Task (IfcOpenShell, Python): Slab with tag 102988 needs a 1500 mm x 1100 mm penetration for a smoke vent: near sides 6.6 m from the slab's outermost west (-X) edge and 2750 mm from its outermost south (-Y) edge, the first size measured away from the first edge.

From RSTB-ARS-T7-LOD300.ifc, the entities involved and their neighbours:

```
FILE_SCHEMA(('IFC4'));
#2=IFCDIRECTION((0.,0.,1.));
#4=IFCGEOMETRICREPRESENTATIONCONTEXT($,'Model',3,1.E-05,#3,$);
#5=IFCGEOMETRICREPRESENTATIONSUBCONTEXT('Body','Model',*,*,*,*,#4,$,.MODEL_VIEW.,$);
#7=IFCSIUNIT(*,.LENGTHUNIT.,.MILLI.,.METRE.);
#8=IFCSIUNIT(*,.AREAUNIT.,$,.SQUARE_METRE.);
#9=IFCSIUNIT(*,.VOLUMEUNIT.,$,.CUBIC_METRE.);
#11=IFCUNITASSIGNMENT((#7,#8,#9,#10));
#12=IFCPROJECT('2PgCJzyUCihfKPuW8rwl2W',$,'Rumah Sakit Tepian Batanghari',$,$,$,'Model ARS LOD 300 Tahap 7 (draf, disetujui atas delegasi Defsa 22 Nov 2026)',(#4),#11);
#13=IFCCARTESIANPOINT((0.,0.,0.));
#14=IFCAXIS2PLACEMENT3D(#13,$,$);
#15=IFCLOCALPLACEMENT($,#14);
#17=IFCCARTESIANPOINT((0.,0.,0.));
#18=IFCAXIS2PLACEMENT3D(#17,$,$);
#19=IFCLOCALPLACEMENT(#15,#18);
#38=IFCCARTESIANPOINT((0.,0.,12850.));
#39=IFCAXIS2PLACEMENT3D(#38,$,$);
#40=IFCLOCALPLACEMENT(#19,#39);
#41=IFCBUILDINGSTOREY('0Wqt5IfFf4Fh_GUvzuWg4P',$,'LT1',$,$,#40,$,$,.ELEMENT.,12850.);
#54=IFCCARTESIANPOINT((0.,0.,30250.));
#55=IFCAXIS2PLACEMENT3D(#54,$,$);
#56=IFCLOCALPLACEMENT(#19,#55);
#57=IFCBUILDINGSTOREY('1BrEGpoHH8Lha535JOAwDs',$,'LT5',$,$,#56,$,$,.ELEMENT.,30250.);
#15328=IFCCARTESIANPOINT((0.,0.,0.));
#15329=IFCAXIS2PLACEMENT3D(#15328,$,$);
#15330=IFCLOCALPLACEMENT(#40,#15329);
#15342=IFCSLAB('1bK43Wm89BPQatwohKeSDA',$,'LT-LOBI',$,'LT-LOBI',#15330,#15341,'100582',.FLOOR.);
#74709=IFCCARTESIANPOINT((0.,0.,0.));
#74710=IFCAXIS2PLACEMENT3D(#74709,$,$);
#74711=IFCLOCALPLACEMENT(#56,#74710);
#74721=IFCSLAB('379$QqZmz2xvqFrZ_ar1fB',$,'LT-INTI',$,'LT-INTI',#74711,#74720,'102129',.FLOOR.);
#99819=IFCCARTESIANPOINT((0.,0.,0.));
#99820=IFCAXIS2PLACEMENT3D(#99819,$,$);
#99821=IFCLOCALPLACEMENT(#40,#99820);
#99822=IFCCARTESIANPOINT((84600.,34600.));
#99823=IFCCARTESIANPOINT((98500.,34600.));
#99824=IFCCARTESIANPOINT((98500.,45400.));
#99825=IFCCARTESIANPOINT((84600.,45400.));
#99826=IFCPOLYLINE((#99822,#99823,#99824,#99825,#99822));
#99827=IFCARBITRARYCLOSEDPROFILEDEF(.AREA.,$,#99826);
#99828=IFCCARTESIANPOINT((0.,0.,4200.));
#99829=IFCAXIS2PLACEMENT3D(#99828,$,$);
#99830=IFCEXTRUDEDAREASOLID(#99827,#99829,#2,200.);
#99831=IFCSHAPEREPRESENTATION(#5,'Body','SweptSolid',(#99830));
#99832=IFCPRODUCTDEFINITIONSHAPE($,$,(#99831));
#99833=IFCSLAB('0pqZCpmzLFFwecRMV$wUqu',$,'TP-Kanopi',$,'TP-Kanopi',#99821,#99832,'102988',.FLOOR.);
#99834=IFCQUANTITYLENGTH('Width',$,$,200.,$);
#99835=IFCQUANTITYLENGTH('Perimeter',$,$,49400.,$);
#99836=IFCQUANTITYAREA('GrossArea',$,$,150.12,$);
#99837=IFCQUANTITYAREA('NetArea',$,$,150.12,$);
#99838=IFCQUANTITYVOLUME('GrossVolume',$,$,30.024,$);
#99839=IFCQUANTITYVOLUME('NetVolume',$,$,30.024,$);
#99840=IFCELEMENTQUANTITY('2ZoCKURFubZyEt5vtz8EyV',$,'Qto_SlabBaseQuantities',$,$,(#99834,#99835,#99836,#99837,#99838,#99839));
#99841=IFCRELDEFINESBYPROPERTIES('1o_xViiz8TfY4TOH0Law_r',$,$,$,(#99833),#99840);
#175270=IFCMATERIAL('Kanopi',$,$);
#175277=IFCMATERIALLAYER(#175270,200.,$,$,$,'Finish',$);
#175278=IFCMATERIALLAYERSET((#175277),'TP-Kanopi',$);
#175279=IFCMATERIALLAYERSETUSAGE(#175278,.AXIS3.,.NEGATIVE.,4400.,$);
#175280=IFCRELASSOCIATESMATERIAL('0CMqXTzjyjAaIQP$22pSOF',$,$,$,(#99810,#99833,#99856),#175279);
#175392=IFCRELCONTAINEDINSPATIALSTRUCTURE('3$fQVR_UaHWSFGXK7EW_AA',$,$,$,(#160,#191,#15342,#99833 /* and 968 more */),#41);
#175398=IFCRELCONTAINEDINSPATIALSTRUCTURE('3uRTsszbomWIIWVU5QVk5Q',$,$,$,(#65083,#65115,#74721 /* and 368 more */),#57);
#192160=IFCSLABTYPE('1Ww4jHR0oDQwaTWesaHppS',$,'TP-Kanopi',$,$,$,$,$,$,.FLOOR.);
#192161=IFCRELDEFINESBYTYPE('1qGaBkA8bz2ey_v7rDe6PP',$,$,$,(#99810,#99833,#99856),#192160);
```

```python
import numpy as np
import ifcopenshell
import ifcopenshell.api.feature
import ifcopenshell.api.geometry
import ifcopenshell.api.pset
import ifcopenshell.api.root
import ifcopenshell.geom
import ifcopenshell.util.element
import ifcopenshell.util.placement
import ifcopenshell.util.representation
import ifcopenshell.util.shape
import ifcopenshell.util.unit

model = ifcopenshell.open("RSTB-ARS-T7-LOD300.ifc")
unit_scale = ifcopenshell.util.unit.calculate_unit_scale(model)
area_scale = ifcopenshell.util.unit.calculate_unit_scale(model, "AREAUNIT")
volume_scale = ifcopenshell.util.unit.calculate_unit_scale(model, "VOLUMEUNIT")
settings = ifcopenshell.geom.settings()


def volume(element):
    """Net volume in cubic metres, openings subtracted."""
    shape = ifcopenshell.geom.create_shape(settings, element)
    return ifcopenshell.util.shape.get_volume(shape.geometry)


slab = model.by_guid("0pqZCpmzLFFwecRMV$wUqu")
before = volume(slab)

# Extent in the slab's own axes, in metres. The edges named are its -X and -Y sides.
slab_shape = ifcopenshell.geom.create_shape(settings, slab)
vertices = ifcopenshell.util.shape.get_vertices(slab_shape.geometry)
x_min, y_min, bottom = vertices.min(axis=0)
top = vertices[:, 2].max()

opening = ifcopenshell.api.root.create_entity(model, ifc_class="IfcOpeningElement", name="Smoke vent opening", predefined_type="OPENING")
context = ifcopenshell.util.representation.get_context(model, "Model", "Body", "MODEL_VIEW")
width, depth = 1.5, 1.1
outline = [(0.0, 0.0), (width, 0.0), (width, depth), (0.0, depth), (0.0, 0.0)]
# Overshoot both faces by 50 mm so the cut is clean.
shape = ifcopenshell.api.geometry.add_slab_representation(
    model, context=context, depth=top - bottom + 0.1, polyline=outline
)
ifcopenshell.api.geometry.assign_representation(model, product=opening, representation=shape)

matrix = ifcopenshell.util.placement.get_local_placement(slab.ObjectPlacement)
matrix[:, 3] = matrix @ np.append(np.array([x_min + 6.6, y_min + 2.75, bottom - 0.05]) / unit_scale, 1.0)
ifcopenshell.api.geometry.edit_object_placement(model, product=opening, matrix=matrix, is_si=False)
ifcopenshell.api.feature.add_feature(model, feature=opening, element=slab)

after = volume(slab)

# Update the slab's stored quantities.
qto = model.by_id(ifcopenshell.util.element.get_pset(slab, "Qto_SlabBaseQuantities", should_inherit=False)["id"])
ifcopenshell.api.pset.edit_qto(model, qto=qto, properties={
    "NetArea": after / (top - bottom) / area_scale,
    "NetVolume": after / volume_scale,
})

print(f"slab volume {before:.3f} -> {after:.3f} m3")

model.write("RSTB-ARS-T7-LOD300_rev.ifc")
```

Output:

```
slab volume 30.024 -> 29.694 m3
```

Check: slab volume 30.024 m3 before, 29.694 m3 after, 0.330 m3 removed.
